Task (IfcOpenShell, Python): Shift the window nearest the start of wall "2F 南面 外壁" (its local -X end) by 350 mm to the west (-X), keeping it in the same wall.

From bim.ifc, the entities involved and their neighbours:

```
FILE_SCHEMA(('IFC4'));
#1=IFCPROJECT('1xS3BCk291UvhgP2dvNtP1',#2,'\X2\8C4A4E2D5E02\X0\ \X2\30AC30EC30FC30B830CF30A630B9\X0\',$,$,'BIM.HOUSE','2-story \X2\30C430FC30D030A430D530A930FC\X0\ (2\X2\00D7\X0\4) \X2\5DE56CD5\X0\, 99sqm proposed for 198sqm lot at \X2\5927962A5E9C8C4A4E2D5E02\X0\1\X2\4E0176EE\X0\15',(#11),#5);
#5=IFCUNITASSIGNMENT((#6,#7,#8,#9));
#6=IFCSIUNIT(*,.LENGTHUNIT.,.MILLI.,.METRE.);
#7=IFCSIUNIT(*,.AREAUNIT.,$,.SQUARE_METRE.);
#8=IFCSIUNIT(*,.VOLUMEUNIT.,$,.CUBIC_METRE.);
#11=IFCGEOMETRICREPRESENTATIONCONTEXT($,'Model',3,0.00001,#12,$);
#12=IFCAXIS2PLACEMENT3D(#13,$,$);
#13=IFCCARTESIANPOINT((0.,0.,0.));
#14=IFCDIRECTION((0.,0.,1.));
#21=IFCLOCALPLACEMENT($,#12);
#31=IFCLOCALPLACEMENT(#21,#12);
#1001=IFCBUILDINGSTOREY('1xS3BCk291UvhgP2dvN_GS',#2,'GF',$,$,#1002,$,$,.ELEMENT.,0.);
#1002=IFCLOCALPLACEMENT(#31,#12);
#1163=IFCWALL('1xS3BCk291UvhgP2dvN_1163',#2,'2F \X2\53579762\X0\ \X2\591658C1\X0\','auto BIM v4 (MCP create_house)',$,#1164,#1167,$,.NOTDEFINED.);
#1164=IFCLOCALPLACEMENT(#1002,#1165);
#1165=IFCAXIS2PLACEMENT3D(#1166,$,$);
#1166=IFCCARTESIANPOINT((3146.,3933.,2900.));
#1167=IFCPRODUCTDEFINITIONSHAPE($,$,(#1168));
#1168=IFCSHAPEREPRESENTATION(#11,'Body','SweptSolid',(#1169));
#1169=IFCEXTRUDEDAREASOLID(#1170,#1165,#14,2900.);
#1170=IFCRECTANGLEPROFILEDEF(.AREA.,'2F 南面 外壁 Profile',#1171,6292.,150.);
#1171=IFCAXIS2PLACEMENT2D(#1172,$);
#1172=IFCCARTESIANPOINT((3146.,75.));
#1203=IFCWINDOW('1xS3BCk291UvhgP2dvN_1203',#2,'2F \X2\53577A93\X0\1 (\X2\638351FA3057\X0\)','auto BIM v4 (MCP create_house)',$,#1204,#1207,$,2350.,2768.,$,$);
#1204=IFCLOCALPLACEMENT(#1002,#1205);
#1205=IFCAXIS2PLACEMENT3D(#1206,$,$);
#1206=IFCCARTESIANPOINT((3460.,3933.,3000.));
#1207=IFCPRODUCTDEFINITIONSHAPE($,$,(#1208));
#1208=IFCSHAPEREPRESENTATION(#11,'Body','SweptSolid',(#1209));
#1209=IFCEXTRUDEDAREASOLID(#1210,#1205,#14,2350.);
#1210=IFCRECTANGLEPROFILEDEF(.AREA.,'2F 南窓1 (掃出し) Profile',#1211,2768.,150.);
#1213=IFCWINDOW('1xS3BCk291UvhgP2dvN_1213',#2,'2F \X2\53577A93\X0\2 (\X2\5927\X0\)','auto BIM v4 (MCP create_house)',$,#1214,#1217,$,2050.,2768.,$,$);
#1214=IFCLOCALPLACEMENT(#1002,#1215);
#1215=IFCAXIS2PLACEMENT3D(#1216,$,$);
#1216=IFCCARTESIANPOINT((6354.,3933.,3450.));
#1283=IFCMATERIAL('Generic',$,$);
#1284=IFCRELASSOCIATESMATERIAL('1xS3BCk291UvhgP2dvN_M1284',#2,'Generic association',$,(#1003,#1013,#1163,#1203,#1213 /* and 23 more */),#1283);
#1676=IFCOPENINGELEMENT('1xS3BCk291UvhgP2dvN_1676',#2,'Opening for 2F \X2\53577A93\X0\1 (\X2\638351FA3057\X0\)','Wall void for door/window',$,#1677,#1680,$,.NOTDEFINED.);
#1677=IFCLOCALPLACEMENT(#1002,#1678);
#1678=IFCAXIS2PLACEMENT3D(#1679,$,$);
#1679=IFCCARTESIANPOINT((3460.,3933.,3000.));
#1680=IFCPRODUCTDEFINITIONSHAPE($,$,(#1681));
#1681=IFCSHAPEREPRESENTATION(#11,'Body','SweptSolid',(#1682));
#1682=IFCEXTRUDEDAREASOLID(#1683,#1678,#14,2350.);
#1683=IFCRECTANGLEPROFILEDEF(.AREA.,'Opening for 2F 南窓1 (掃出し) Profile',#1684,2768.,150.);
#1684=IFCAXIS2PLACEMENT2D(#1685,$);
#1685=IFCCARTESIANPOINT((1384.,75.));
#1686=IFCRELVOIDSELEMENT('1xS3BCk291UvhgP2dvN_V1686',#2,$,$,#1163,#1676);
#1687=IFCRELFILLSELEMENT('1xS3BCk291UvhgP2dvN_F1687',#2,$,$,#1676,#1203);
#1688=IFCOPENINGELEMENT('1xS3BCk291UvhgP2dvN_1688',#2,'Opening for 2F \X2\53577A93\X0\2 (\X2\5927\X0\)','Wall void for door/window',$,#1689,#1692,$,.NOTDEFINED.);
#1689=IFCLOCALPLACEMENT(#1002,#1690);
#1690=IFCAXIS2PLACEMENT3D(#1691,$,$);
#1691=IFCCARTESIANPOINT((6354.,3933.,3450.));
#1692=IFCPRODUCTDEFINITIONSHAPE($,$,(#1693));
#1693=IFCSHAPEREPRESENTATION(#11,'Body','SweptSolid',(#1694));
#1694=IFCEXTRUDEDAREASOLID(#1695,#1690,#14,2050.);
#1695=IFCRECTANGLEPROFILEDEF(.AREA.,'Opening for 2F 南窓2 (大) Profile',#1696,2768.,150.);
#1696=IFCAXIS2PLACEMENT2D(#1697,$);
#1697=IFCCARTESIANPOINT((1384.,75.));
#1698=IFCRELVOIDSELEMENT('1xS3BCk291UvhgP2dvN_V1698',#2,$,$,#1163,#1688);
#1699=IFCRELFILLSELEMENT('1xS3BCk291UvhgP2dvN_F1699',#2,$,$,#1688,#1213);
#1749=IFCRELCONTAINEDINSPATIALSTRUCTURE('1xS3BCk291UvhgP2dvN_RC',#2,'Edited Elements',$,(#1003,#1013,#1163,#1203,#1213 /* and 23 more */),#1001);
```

```python
import ifcopenshell
import ifcopenshell.api.geometry
import ifcopenshell.util.placement
import ifcopenshell.util.unit

model = ifcopenshell.open("bim.ifc")
unit_scale = ifcopenshell.util.unit.calculate_unit_scale(model)

window = model.by_id(1203)
opening = window.FillsVoids[0].RelatingOpeningElement
wall = opening.VoidsElements[0].RelatingBuildingElement

wall_matrix = ifcopenshell.util.placement.get_local_placement(wall.ObjectPlacement)
shift = wall_matrix[:3, 0] * -0.35 / unit_scale
before = ifcopenshell.util.placement.get_local_placement(window.ObjectPlacement)[:3, 3].copy()

# The window is not placed relative to its opening, so move both.
for product in (opening, window):
    matrix = ifcopenshell.util.placement.get_local_placement(product.ObjectPlacement)
    matrix[:3, 3] += shift
    ifcopenshell.api.geometry.edit_object_placement(model, product=product, matrix=matrix, is_si=False)

after = ifcopenshell.util.placement.get_local_placement(window.ObjectPlacement)[:3, 3]
print("window moved by", (after - before).round(3) + 0.0)

model.write("bim_edited.ifc")
```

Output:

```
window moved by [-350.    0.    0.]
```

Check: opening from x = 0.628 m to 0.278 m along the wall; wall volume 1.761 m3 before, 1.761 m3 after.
